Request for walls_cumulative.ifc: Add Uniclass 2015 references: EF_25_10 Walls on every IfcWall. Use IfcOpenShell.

First a look at what the model holds.

```python
import ifcopenshell

model = ifcopenshell.open("walls_cumulative.ifc")
print(model.schema)
print("classifications:", [c.Name for c in model.by_type("IfcClassification")])
for ifc_class in ("IfcDoor", "IfcRoof", "IfcStair", "IfcWall", "IfcWindow"):
    print(ifc_class, len(model.by_type(ifc_class)))
```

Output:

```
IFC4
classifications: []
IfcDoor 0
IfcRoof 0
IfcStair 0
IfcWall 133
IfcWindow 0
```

```python
import ifcopenshell
import ifcopenshell.api.classification

model = ifcopenshell.open("walls_cumulative.ifc")

system = ifcopenshell.api.classification.add_classification(model, classification="Uniclass 2015")

codes = {
    "IfcWall": ("EF_25_10", "Walls"),
}
for ifc_class, (code, name) in codes.items():
    products = model.by_type(ifc_class)
    ifcopenshell.api.classification.add_reference(
        model, products=products, classification=system, identification=code, name=name
    )
    print(code, len(products))

model.write("walls_cumulative-out.ifc")
```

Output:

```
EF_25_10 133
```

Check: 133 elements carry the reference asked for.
